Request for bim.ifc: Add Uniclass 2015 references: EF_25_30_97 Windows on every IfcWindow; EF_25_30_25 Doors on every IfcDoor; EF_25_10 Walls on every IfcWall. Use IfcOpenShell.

First a look at what the model holds.

```python
import ifcopenshell

model = ifcopenshell.open("bim.ifc")
print(model.schema)
print("classifications:", [c.Name for c in model.by_type("IfcClassification")])
for ifc_class in ("IfcDoor", "IfcRoof", "IfcStair", "IfcWall", "IfcWindow"):
    print(ifc_class, len(model.by_type(ifc_class)))
```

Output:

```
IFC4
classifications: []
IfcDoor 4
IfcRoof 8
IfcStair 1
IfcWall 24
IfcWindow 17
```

```python
import ifcopenshell
import ifcopenshell.api.classification

model = ifcopenshell.open("bim.ifc")

system = ifcopenshell.api.classification.add_classification(model, classification="Uniclass 2015")

codes = {
    "IfcWindow": ("EF_25_30_97", "Windows"),
    "IfcDoor": ("EF_25_30_25", "Doors"),
    "IfcWall": ("EF_25_10", "Walls"),
}
for ifc_class, (code, name) in codes.items():
    products = model.by_type(ifc_class)
    ifcopenshell.api.classification.add_reference(
        model, products=products, classification=system, identification=code, name=name
    )
    print(code, len(products))

model.write("bim_rev.ifc")
```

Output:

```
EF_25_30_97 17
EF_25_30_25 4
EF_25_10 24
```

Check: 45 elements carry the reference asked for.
